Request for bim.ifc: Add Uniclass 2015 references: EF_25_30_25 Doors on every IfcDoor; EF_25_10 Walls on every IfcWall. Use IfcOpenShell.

First a look at what the model holds.

```python
import ifcopenshell

model = ifcopenshell.open("bim.ifc")
print(model.schema)
print("classifications:", [c.Name for c in model.by_type("IfcClassification")])
for ifc_class in ("IfcDoor", "IfcRoof", "IfcStair", "IfcWall", "IfcWindow"):
    print(ifc_class, len(model.by_type(ifc_class)))
```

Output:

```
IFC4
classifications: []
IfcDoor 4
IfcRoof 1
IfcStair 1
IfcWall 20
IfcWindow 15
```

```python
import ifcopenshell
import ifcopenshell.api.classification

model = ifcopenshell.open("bim.ifc")

system = ifcopenshell.api.classification.add_classification(model, classification="Uniclass 2015")

codes = {
    "IfcDoor": ("EF_25_30_25", "Doors"),
    "IfcWall": ("EF_25_10", "Walls"),
}
for ifc_class, (code, name) in codes.items():
    products = model.by_type(ifc_class)
    ifcopenshell.api.classification.add_reference(
        model, products=products, classification=system, identification=code, name=name
    )
    print(code, len(products))

model.write("bim_updated.ifc")
```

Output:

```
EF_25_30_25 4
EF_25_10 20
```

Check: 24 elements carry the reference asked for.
